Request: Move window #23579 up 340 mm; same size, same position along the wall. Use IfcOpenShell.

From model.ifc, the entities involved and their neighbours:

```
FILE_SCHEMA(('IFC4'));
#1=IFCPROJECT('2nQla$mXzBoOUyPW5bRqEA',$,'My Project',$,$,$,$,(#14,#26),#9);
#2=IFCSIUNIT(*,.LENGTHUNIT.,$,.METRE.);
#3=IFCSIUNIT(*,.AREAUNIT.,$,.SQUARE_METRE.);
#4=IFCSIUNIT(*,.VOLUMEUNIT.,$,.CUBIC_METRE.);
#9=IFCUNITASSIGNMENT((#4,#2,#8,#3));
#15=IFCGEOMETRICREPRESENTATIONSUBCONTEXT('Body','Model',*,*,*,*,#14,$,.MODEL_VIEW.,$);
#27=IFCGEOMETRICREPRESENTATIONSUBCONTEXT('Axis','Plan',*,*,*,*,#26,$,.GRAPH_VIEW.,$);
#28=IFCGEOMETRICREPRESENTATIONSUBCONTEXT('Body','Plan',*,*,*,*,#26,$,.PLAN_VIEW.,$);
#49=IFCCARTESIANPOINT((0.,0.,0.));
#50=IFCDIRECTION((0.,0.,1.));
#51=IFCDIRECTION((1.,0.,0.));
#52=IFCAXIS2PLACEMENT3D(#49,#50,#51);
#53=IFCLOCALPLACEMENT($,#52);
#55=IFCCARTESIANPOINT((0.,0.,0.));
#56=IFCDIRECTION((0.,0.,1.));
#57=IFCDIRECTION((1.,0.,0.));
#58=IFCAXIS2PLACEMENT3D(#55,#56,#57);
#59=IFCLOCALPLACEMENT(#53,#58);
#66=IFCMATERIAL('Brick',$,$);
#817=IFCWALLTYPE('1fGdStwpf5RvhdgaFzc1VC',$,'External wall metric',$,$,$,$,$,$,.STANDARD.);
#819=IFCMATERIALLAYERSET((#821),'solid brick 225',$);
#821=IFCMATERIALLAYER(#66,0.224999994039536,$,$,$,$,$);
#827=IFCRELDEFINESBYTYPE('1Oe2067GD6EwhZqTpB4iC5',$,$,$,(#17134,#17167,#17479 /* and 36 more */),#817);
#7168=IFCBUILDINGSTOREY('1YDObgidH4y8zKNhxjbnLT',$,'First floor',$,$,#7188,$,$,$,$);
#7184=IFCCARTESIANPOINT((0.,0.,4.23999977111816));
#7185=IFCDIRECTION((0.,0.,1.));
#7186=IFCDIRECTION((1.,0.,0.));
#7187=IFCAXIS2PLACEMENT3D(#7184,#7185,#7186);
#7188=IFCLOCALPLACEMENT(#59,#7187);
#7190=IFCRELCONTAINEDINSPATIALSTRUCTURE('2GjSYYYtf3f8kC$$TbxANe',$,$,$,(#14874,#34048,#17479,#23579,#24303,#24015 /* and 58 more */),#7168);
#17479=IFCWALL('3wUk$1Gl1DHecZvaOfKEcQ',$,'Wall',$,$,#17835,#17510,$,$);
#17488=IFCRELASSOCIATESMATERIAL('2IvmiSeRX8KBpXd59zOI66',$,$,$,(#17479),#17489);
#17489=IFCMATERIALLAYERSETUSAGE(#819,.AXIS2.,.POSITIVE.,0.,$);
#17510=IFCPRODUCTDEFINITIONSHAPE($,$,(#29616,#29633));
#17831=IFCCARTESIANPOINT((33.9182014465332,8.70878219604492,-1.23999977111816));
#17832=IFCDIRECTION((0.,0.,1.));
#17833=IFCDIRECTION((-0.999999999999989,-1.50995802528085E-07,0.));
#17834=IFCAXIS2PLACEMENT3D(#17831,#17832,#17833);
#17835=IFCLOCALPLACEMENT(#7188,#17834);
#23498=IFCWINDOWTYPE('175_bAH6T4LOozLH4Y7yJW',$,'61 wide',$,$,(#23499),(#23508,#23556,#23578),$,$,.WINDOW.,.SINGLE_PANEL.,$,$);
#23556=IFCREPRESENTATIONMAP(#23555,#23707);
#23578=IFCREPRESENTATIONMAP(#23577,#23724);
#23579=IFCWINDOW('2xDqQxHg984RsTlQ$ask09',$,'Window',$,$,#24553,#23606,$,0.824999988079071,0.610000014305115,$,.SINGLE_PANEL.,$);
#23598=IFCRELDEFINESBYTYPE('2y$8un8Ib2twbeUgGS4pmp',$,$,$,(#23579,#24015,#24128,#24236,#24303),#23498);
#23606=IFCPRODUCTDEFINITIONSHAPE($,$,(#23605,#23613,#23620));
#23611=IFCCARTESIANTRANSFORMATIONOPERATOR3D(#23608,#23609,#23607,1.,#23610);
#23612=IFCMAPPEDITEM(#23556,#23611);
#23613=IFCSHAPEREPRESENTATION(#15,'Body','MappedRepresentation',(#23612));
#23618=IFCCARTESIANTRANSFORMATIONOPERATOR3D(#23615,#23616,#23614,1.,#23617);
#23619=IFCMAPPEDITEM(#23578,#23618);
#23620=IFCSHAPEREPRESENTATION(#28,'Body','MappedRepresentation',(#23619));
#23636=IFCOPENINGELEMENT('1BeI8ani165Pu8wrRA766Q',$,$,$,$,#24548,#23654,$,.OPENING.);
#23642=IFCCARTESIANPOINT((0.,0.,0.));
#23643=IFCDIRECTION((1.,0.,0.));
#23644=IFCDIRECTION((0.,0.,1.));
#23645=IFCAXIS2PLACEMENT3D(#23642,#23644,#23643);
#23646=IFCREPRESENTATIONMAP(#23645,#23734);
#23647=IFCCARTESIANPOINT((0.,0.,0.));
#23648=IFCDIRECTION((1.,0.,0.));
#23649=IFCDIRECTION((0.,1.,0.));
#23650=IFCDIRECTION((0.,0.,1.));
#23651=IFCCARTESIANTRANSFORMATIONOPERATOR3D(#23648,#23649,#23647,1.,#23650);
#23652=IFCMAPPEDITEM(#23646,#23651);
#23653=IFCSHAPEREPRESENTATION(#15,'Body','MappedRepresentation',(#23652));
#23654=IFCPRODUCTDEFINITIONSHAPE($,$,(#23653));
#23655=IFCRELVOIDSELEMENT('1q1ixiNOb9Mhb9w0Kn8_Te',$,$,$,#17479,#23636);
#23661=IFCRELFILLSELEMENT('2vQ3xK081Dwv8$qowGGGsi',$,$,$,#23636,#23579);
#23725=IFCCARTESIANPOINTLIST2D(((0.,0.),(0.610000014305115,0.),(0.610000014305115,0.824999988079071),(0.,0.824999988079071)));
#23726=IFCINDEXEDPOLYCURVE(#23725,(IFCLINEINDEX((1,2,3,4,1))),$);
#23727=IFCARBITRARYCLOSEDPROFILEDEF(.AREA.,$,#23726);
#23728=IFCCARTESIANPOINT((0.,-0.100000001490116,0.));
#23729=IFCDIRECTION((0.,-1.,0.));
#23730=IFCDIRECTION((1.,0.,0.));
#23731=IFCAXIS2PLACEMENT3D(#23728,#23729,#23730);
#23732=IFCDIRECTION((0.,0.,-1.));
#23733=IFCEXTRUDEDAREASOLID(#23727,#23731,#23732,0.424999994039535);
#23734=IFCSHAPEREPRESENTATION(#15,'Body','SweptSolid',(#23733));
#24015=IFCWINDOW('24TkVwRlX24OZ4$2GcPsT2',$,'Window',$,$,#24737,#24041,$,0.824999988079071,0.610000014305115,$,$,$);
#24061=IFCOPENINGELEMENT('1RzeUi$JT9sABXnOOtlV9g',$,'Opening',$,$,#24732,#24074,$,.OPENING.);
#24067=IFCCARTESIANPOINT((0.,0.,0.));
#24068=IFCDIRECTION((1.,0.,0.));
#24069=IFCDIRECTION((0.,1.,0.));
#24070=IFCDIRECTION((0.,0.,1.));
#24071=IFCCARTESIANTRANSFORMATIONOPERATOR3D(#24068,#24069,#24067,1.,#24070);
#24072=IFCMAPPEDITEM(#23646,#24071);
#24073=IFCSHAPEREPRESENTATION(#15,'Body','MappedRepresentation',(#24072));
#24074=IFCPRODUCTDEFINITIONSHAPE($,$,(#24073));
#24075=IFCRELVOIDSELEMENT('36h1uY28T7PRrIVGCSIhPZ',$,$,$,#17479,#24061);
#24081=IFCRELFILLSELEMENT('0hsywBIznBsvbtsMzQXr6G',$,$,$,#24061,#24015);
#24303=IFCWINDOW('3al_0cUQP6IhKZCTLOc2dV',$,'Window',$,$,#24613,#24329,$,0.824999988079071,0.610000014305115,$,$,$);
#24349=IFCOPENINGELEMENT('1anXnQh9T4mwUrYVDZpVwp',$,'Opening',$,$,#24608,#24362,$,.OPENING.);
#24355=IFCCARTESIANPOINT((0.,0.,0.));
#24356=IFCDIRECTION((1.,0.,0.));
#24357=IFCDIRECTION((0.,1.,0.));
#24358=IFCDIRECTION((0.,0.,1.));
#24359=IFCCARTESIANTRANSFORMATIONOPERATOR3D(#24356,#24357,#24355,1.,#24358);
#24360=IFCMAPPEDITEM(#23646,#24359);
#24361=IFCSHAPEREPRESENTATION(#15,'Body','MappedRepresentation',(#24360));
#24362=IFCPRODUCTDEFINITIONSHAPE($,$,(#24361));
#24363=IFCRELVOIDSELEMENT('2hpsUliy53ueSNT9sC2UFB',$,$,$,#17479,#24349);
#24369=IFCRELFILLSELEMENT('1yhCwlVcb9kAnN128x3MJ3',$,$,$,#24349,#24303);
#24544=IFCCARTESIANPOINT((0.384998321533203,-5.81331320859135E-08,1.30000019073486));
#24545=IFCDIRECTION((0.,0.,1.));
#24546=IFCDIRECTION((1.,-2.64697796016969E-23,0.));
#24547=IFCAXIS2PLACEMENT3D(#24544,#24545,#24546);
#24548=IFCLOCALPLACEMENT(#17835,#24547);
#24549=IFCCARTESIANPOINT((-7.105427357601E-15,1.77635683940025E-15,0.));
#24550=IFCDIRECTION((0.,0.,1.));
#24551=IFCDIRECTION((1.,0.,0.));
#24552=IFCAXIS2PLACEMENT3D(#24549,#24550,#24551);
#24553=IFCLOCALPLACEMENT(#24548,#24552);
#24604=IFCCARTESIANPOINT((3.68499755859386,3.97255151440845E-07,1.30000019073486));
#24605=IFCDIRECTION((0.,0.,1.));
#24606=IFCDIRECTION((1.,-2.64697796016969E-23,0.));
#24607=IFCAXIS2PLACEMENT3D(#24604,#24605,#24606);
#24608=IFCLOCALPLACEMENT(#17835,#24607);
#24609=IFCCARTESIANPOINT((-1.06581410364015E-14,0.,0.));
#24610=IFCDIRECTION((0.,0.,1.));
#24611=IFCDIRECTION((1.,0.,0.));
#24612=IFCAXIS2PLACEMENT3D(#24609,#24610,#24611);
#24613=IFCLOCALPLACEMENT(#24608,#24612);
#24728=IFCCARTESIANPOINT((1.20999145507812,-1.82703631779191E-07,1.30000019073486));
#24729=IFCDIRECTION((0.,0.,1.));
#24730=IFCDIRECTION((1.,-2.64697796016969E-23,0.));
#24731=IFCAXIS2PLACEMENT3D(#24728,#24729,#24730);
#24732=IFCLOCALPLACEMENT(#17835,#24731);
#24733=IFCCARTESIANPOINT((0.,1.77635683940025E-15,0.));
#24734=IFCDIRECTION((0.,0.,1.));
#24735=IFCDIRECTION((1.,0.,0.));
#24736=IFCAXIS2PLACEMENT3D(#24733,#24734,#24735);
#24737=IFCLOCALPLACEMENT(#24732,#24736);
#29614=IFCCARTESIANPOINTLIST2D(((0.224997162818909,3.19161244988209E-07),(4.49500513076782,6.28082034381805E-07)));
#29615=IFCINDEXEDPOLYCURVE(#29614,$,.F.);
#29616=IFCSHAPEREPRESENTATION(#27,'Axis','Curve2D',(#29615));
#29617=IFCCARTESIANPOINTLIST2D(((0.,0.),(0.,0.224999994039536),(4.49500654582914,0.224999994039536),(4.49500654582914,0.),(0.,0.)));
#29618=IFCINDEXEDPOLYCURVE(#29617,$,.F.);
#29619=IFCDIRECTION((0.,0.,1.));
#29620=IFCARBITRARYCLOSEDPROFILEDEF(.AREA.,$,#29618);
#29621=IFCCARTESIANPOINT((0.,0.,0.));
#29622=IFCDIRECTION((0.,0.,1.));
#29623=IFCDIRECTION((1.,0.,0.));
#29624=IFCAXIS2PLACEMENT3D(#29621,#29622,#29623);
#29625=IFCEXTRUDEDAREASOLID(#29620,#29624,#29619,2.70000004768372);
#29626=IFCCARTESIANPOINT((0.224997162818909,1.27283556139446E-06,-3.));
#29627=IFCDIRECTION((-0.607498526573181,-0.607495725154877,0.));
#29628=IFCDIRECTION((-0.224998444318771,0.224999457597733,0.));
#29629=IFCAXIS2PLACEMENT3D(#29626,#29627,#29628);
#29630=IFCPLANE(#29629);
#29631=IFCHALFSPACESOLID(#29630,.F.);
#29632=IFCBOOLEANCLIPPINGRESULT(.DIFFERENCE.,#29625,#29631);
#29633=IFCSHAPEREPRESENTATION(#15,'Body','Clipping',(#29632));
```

```python
import numpy as np
import ifcopenshell
import ifcopenshell.api.geometry
import ifcopenshell.util.placement
import ifcopenshell.util.unit

model = ifcopenshell.open("model.ifc")
unit_scale = ifcopenshell.util.unit.calculate_unit_scale(model)

window = model.by_id(23579)
opening = window.FillsVoids[0].RelatingOpeningElement
dz = 0.34 / unit_scale

shift = np.array([0.0, 0.0, dz])
# The window is placed relative to its opening, so it follows when the opening moves.
matrix = ifcopenshell.util.placement.get_local_placement(opening.ObjectPlacement)
matrix[:3, 3] += shift
ifcopenshell.api.geometry.edit_object_placement(
    model, product=opening, matrix=matrix, is_si=False, should_transform_children=True
)

print(f"moved by {dz * unit_scale:+.3f} m")

model.write("model_updated.ifc")
```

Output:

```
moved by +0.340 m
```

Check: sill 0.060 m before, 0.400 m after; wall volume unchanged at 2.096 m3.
